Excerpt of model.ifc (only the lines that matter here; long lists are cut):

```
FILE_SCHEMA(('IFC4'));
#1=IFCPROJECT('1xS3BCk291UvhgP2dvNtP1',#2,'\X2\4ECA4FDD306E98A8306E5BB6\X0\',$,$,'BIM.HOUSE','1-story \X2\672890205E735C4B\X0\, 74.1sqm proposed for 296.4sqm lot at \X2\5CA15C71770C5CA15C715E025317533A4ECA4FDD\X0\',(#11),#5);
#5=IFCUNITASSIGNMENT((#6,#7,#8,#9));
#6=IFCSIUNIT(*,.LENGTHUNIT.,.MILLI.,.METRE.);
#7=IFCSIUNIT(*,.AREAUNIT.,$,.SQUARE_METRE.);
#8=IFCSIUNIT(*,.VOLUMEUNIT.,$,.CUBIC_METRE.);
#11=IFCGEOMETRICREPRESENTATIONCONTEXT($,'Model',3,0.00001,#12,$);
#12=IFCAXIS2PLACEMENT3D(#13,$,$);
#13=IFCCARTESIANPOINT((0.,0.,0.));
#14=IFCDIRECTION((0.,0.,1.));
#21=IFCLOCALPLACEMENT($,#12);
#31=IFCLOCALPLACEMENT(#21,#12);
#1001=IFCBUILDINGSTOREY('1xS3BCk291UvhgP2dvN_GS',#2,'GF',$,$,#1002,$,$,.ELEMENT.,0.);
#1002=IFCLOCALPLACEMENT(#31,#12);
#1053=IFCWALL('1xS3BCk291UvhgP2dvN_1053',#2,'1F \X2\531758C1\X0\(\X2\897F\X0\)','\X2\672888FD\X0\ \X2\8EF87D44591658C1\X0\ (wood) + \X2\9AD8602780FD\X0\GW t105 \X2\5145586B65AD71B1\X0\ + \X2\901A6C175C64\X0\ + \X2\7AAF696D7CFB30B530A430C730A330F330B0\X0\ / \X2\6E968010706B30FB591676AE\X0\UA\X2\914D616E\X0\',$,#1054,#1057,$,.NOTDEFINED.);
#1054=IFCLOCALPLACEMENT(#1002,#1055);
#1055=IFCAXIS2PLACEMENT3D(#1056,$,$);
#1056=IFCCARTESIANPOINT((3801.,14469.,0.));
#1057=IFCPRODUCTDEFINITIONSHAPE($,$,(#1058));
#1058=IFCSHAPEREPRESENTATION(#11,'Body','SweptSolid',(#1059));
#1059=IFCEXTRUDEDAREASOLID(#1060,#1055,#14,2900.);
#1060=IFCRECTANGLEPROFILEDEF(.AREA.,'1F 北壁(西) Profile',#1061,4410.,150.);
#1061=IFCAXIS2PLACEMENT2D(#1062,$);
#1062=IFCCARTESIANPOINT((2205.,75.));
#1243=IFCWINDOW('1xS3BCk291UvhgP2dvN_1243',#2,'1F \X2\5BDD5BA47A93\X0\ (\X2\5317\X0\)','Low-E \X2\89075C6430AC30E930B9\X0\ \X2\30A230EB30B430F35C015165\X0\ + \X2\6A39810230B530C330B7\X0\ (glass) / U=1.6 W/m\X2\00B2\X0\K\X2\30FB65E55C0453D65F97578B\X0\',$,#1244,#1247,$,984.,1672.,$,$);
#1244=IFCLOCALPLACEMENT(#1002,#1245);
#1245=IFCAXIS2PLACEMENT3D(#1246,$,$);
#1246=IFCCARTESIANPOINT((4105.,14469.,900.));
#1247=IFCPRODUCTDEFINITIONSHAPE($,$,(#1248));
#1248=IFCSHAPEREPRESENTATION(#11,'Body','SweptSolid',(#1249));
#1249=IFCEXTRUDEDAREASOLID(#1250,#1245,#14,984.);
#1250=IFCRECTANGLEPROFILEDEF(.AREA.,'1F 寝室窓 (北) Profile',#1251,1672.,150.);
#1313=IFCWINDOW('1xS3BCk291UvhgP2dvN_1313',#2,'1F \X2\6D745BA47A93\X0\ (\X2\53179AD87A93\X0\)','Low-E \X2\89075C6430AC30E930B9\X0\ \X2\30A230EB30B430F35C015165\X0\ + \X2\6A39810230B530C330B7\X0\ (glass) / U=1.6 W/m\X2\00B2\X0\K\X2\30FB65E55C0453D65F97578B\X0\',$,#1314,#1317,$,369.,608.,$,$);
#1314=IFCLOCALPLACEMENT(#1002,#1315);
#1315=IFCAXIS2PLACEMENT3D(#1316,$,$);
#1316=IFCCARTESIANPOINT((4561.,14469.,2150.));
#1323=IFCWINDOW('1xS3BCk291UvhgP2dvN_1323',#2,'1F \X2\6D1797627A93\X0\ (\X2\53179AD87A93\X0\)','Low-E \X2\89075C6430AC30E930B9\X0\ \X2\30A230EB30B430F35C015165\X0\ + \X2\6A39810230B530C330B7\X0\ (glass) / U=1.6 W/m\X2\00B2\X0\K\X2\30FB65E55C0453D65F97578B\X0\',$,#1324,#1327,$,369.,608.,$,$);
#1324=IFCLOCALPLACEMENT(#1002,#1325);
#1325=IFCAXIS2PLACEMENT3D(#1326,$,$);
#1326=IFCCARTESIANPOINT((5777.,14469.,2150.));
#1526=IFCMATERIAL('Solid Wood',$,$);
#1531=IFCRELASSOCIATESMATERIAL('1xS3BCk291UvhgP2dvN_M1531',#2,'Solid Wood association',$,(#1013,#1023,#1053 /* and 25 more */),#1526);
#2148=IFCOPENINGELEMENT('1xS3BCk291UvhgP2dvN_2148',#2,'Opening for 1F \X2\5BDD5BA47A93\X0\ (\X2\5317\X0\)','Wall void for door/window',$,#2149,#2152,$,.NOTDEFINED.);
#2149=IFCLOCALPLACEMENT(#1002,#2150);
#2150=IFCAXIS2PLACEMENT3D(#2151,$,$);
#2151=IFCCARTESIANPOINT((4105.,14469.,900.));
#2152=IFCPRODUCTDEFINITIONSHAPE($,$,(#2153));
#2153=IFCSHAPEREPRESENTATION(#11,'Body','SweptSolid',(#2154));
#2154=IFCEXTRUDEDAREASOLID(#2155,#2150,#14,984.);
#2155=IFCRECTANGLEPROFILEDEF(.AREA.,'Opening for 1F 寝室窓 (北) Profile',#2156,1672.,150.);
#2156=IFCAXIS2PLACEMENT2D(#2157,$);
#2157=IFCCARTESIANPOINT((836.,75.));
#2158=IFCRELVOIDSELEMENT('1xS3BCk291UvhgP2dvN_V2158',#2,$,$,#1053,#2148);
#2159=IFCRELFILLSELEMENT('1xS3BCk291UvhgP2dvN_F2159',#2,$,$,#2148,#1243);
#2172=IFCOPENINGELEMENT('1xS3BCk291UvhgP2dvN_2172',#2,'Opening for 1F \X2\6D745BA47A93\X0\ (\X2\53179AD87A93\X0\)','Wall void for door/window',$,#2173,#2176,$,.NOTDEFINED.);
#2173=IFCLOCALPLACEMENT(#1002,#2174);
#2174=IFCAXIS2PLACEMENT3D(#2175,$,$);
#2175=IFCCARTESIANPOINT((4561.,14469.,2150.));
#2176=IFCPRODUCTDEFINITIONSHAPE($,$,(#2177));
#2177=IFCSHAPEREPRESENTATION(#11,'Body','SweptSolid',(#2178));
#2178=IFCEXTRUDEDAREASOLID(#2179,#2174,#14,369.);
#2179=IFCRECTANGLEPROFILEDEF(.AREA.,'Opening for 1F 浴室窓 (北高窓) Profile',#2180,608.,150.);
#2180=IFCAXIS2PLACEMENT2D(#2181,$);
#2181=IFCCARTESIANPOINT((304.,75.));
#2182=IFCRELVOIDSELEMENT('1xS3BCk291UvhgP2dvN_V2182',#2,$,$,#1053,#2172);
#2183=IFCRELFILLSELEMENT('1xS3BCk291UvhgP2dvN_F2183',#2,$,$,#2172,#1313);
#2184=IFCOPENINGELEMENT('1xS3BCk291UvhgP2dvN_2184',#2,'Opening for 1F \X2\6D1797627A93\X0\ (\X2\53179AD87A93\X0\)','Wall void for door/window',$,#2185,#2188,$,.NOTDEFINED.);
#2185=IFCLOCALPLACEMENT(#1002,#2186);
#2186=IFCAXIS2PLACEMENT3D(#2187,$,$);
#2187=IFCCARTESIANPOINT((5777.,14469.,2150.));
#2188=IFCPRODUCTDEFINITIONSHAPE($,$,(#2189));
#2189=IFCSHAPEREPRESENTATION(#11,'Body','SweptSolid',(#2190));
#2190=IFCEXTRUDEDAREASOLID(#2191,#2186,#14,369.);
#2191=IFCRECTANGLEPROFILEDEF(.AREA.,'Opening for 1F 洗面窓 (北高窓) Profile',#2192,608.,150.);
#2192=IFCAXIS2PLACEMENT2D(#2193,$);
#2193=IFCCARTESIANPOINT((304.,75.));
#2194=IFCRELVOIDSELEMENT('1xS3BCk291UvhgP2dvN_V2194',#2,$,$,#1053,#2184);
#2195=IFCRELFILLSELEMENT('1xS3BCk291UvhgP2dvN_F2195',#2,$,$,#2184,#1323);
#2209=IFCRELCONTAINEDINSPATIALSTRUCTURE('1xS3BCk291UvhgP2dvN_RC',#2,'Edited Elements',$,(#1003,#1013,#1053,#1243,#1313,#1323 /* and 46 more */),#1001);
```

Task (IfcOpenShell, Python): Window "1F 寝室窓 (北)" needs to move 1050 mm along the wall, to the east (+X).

```python
import ifcopenshell
import ifcopenshell.api.geometry
import ifcopenshell.util.placement
import ifcopenshell.util.unit

model = ifcopenshell.open("model.ifc")
unit_scale = ifcopenshell.util.unit.calculate_unit_scale(model)

window = model.by_id(1243)
opening = window.FillsVoids[0].RelatingOpeningElement
wall = opening.VoidsElements[0].RelatingBuildingElement

wall_matrix = ifcopenshell.util.placement.get_local_placement(wall.ObjectPlacement)
shift = wall_matrix[:3, 0] * 1.05 / unit_scale
before = ifcopenshell.util.placement.get_local_placement(window.ObjectPlacement)[:3, 3].copy()

# The window is not placed relative to its opening, so move both.
for product in (opening, window):
    matrix = ifcopenshell.util.placement.get_local_placement(product.ObjectPlacement)
    matrix[:3, 3] += shift
    ifcopenshell.api.geometry.edit_object_placement(model, product=product, matrix=matrix, is_si=False)

after = ifcopenshell.util.placement.get_local_placement(window.ObjectPlacement)[:3, 3]
print("window moved by", (after - before).round(3) + 0.0)

model.write("model_v2.ifc")
```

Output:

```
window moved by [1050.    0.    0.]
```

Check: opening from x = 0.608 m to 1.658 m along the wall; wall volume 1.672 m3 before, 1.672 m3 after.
